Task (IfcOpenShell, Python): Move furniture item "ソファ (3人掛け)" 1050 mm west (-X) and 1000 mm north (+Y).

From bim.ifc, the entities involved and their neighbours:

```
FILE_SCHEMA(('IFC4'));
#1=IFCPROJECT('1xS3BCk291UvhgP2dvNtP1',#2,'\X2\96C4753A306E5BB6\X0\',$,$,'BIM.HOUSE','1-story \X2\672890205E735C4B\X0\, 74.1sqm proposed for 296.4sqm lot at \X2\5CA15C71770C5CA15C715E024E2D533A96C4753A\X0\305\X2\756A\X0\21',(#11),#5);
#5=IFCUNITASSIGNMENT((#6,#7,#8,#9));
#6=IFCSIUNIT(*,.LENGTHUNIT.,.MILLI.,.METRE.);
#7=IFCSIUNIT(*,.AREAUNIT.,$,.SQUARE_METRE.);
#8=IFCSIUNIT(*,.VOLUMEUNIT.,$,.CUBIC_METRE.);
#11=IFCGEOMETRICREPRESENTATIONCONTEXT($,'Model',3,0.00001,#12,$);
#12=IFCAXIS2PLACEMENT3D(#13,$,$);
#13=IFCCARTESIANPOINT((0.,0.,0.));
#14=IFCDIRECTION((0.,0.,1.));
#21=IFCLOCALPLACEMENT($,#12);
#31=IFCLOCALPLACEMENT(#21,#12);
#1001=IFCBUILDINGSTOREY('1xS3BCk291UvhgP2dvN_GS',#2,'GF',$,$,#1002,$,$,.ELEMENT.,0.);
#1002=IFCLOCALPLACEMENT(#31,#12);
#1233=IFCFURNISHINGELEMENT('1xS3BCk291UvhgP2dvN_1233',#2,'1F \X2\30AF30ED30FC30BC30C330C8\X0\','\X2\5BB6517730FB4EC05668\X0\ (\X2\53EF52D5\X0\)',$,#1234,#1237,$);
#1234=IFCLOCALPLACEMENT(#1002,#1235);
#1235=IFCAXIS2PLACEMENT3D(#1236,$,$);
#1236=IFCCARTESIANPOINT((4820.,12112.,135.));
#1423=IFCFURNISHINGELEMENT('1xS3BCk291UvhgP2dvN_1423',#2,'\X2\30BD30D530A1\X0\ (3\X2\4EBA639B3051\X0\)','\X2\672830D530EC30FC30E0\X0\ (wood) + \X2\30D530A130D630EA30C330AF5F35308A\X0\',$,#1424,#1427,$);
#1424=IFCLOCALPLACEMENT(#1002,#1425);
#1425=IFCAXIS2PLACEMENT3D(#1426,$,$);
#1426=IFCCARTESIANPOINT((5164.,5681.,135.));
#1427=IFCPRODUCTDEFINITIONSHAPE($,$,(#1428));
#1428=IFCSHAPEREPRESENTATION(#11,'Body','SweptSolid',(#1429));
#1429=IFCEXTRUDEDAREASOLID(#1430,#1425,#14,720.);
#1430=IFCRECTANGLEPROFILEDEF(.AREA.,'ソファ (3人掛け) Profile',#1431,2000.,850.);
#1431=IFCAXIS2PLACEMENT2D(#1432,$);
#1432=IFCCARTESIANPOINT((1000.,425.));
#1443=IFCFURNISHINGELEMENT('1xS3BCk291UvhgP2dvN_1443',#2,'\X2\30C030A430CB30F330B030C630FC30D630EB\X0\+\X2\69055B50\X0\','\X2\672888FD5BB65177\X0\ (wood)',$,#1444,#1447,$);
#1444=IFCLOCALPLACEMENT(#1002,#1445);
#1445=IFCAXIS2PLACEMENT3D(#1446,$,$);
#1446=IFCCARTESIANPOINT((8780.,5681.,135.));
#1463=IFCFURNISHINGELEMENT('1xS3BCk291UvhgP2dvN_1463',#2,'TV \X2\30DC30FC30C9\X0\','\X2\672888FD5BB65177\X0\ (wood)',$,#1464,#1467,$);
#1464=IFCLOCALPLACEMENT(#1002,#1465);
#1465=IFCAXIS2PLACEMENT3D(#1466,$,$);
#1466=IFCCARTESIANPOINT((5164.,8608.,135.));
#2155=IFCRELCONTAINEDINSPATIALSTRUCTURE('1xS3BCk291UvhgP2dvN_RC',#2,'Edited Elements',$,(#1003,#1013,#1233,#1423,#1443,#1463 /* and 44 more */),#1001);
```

```python
import ifcopenshell
import ifcopenshell.api.geometry
import ifcopenshell.util.placement
import ifcopenshell.util.unit

model = ifcopenshell.open("bim.ifc")
unit_scale = ifcopenshell.util.unit.calculate_unit_scale(model)

item = model.by_id(1423)
matrix = ifcopenshell.util.placement.get_local_placement(item.ObjectPlacement)
matrix[0, 3] -= 1.05 / unit_scale
matrix[1, 3] += 1 / unit_scale
ifcopenshell.api.geometry.edit_object_placement(model, product=item, matrix=matrix, is_si=False)

print(ifcopenshell.util.placement.get_local_placement(item.ObjectPlacement).round(3) + 0.0)

model.write("bim-out.ifc")
```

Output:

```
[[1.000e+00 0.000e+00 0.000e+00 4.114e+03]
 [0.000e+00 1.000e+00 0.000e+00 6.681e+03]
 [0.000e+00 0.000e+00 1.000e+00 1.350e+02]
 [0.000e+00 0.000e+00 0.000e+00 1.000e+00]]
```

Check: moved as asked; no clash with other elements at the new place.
